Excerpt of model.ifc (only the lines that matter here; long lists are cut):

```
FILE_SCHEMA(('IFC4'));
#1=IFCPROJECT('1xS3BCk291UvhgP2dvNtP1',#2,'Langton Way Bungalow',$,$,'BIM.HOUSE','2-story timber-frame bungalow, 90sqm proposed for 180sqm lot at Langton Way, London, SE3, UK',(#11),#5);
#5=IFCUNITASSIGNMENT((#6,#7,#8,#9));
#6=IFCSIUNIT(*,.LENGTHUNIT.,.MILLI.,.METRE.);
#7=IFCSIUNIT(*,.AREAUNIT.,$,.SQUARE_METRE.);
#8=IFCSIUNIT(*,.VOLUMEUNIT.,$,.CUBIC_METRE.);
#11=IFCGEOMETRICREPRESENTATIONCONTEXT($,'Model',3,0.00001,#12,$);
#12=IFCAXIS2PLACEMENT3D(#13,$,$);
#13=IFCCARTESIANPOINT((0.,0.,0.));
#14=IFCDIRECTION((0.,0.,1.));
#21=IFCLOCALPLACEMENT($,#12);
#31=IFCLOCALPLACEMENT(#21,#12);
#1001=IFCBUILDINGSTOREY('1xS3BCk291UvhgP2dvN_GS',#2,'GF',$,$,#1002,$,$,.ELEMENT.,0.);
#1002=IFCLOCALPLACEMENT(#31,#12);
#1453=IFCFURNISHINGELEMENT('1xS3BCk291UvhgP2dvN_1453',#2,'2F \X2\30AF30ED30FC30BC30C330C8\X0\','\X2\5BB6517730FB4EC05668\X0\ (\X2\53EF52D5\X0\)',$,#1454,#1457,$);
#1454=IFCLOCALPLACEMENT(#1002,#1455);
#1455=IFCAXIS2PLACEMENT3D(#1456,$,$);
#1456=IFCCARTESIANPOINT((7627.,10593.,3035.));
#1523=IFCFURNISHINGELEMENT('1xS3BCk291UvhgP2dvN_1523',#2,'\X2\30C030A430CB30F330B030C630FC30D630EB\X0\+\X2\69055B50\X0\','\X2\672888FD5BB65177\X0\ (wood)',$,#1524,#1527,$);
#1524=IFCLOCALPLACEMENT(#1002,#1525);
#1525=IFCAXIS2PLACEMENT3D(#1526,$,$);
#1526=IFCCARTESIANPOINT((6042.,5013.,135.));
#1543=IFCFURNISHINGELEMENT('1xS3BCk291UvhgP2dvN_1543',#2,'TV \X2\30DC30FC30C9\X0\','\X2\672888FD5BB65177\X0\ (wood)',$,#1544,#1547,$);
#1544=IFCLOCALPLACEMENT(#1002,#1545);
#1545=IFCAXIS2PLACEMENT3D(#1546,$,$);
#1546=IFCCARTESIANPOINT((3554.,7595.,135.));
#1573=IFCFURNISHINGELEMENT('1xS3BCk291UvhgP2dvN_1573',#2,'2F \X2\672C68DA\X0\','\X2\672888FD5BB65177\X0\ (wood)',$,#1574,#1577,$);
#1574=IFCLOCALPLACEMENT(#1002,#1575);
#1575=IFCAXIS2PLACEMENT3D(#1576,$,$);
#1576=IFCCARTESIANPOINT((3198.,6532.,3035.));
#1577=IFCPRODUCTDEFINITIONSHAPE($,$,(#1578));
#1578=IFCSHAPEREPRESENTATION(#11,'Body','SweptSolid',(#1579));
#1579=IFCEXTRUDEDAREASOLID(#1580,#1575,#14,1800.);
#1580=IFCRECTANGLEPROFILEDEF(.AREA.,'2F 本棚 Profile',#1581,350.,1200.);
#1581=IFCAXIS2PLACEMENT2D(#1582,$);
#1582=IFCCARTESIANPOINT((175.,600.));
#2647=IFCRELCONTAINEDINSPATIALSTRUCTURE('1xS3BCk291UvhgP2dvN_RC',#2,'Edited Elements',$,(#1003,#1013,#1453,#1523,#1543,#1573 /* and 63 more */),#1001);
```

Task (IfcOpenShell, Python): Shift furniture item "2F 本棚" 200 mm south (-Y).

```python
import ifcopenshell
import ifcopenshell.api.geometry
import ifcopenshell.util.placement
import ifcopenshell.util.unit

model = ifcopenshell.open("model.ifc")
unit_scale = ifcopenshell.util.unit.calculate_unit_scale(model)

item = model.by_guid("1xS3BCk291UvhgP2dvN_1573")
matrix = ifcopenshell.util.placement.get_local_placement(item.ObjectPlacement)
matrix[1, 3] -= 0.2 / unit_scale
ifcopenshell.api.geometry.edit_object_placement(model, product=item, matrix=matrix, is_si=False)

print(ifcopenshell.util.placement.get_local_placement(item.ObjectPlacement).round(3) + 0.0)

model.write("model_edited.ifc")
```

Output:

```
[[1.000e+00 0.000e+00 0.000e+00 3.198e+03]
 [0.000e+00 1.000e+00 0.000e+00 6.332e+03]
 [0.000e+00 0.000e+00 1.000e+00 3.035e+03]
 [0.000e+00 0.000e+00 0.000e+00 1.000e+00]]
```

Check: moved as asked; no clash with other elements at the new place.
